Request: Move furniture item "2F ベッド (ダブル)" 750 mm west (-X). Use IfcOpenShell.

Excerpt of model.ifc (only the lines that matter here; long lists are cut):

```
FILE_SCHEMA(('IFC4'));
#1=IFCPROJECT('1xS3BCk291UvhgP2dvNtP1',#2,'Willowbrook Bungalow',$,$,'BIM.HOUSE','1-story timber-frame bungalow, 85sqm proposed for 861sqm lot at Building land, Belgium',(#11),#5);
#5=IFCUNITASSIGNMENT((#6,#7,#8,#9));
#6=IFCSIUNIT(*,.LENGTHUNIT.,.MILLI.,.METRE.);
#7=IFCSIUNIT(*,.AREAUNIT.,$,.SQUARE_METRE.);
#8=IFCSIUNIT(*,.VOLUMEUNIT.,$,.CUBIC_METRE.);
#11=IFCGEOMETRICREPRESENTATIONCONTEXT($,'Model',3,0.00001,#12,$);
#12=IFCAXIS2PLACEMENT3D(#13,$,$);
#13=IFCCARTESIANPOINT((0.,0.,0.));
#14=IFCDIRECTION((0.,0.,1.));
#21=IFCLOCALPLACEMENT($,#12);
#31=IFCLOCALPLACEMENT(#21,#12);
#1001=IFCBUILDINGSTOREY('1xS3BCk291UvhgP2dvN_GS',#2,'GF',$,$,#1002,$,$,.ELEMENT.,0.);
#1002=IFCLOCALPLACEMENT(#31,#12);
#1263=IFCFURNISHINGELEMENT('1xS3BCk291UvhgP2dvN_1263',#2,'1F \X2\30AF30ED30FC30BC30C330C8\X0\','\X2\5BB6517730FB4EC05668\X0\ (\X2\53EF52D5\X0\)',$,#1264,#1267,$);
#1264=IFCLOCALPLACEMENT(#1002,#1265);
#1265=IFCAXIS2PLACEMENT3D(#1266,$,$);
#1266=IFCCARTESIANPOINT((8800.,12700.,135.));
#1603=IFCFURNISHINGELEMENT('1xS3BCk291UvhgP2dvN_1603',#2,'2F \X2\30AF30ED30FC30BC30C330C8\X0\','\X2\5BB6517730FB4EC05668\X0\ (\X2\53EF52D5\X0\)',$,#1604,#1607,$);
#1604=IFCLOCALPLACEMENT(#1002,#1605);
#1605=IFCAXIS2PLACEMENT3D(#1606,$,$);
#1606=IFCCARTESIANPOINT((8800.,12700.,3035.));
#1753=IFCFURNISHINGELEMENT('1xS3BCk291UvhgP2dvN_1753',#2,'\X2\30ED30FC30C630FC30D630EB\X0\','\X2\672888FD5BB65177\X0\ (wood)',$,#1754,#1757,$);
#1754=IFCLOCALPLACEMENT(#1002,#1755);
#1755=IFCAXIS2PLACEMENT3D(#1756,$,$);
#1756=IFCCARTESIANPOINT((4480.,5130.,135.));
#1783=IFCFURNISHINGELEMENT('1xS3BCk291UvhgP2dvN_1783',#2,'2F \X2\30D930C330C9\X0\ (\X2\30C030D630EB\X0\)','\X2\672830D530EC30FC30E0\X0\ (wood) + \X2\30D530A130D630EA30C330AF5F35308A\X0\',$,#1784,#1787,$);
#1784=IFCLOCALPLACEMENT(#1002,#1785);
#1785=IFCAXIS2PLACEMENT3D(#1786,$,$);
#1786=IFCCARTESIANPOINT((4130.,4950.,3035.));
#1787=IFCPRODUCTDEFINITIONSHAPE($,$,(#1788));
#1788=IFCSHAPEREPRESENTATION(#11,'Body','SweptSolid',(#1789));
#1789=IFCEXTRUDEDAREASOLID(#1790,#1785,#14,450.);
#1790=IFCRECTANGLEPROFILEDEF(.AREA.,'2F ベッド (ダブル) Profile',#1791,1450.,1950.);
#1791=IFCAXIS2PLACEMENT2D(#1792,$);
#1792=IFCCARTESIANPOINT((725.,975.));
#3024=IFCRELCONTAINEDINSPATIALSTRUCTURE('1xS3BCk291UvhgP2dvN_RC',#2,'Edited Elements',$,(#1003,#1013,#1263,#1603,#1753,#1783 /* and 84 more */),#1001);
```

```python
import ifcopenshell
import ifcopenshell.api.geometry
import ifcopenshell.util.placement

model = ifcopenshell.open("model.ifc")

item = model.by_guid("1xS3BCk291UvhgP2dvN_1783")
matrix = ifcopenshell.util.placement.get_local_placement(item.ObjectPlacement)
matrix[0, 3] -= 750.0
ifcopenshell.api.geometry.edit_object_placement(model, product=item, matrix=matrix, is_si=False)

print(ifcopenshell.util.placement.get_local_placement(item.ObjectPlacement).round(3) + 0.0)

model.write("model_rev.ifc")
```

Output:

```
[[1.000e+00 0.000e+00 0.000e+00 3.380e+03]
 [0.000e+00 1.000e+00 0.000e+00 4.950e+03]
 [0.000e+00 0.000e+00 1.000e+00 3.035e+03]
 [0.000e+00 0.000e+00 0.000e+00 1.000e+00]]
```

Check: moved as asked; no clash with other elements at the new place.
